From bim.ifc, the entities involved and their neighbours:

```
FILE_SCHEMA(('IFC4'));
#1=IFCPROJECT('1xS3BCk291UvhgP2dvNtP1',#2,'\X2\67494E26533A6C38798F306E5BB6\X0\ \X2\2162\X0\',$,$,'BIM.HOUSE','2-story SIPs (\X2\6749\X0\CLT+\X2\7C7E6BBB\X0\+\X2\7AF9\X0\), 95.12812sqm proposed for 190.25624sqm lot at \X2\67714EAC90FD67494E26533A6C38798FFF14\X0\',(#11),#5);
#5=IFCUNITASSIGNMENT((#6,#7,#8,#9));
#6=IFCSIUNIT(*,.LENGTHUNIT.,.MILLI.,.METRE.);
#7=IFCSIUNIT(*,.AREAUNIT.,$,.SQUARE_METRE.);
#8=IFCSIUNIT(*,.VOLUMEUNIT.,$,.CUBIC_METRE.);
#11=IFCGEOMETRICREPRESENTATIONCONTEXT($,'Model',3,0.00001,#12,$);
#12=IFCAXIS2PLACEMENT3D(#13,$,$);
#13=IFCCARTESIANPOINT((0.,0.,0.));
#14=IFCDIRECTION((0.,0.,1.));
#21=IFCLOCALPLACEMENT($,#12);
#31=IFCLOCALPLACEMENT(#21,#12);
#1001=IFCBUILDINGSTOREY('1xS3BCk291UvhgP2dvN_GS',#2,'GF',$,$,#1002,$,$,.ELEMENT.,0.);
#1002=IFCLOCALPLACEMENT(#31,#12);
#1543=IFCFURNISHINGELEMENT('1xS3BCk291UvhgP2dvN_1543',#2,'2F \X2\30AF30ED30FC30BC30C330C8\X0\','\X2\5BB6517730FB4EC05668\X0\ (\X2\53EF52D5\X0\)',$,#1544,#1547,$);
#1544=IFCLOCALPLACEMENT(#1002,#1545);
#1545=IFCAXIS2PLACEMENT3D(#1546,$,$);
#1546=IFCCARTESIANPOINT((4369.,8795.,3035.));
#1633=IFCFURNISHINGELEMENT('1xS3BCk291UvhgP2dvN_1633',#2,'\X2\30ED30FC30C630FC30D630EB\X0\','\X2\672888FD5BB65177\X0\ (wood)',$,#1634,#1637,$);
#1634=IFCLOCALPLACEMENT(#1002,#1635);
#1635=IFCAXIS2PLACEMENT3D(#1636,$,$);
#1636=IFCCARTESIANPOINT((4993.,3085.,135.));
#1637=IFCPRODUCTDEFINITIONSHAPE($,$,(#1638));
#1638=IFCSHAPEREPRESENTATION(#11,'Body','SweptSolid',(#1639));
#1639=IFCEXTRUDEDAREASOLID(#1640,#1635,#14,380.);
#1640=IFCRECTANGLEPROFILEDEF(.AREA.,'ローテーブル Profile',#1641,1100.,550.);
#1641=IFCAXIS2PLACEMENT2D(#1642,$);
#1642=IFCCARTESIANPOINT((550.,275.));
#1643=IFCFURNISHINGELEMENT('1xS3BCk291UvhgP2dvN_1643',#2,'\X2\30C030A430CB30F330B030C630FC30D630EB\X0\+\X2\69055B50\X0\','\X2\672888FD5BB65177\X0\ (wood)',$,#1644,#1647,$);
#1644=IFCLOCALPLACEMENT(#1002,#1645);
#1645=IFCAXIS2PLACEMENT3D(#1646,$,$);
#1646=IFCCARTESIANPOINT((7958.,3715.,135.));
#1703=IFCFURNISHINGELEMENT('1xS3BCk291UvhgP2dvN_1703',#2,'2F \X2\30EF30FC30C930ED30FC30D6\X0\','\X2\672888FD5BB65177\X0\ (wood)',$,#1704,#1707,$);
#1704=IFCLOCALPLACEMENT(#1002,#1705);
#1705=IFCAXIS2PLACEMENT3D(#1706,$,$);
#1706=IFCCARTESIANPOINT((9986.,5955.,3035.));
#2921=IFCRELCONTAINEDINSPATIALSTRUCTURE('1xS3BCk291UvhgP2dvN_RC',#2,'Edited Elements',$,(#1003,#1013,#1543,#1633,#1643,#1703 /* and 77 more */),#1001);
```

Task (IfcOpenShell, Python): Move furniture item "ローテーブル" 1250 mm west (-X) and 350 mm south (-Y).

```python
import ifcopenshell
import ifcopenshell.api.geometry
import ifcopenshell.util.placement

model = ifcopenshell.open("bim.ifc")

item = model.by_guid("1xS3BCk291UvhgP2dvN_1633")
matrix = ifcopenshell.util.placement.get_local_placement(item.ObjectPlacement)
matrix[0, 3] -= 1250.0
matrix[1, 3] -= 350.0
ifcopenshell.api.geometry.edit_object_placement(model, product=item, matrix=matrix, is_si=False)

print(ifcopenshell.util.placement.get_local_placement(item.ObjectPlacement).round(3) + 0.0)

model.write("bim-out.ifc")
```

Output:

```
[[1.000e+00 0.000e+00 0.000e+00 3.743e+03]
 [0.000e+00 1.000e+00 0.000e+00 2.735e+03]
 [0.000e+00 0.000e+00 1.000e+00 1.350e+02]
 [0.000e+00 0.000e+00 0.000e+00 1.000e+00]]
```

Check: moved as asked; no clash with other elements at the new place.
